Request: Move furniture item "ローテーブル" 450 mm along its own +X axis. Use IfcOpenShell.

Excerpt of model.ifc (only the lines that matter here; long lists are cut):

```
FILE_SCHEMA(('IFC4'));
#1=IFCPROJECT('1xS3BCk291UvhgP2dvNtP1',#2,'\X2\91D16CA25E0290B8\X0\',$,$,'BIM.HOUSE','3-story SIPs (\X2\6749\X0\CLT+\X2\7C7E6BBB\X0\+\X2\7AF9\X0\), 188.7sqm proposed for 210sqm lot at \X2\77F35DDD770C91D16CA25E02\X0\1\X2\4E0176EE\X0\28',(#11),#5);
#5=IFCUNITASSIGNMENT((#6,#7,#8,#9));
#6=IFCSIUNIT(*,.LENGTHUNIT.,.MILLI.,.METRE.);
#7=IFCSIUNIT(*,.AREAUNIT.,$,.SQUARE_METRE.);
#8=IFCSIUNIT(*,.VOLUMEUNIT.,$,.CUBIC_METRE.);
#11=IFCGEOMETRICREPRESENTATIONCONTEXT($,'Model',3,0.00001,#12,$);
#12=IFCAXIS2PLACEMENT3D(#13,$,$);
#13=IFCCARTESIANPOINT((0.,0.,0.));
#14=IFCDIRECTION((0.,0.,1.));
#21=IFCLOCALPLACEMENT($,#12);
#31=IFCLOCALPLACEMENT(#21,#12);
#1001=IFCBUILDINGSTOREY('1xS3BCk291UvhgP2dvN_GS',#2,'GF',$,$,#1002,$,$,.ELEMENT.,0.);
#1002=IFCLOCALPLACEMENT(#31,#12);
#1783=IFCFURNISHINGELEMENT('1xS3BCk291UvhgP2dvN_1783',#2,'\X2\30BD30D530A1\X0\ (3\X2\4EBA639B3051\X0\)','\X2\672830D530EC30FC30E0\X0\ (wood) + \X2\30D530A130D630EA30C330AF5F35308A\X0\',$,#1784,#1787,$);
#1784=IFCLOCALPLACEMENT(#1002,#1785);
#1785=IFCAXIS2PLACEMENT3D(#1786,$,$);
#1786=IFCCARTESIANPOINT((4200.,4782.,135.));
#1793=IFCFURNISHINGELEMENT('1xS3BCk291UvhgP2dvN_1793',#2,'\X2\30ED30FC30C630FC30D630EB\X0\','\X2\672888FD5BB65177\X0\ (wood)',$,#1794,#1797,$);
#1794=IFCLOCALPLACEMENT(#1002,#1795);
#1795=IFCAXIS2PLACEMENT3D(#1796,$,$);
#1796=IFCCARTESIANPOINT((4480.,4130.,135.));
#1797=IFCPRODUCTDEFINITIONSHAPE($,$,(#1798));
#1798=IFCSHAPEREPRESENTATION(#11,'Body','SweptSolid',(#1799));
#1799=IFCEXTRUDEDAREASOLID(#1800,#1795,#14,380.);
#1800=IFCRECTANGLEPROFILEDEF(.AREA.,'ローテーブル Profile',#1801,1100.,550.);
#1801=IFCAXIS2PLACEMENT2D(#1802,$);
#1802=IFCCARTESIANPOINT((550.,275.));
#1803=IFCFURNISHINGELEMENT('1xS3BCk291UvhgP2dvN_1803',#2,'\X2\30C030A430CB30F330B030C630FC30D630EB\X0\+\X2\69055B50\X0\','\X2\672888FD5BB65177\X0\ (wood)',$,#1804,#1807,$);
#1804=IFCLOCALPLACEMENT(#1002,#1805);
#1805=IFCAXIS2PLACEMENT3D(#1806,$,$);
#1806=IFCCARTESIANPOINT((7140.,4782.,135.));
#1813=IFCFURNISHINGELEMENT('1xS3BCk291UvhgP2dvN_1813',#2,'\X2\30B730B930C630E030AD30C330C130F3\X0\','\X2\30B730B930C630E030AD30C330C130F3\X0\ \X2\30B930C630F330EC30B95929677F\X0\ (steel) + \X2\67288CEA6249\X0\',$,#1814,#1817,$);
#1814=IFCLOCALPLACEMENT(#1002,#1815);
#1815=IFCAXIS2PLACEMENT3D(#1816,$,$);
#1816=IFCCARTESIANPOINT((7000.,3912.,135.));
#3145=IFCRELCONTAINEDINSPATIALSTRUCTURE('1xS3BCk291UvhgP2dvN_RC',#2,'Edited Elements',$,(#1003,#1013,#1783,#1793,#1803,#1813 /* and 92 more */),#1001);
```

```python
import ifcopenshell
import ifcopenshell.api.geometry
import ifcopenshell.util.placement

model = ifcopenshell.open("model.ifc")

item = model.by_guid("1xS3BCk291UvhgP2dvN_1793")
matrix = ifcopenshell.util.placement.get_local_placement(item.ObjectPlacement)
matrix[:3, 3] += matrix[:3, 0] * 450.0
ifcopenshell.api.geometry.edit_object_placement(model, product=item, matrix=matrix, is_si=False)

print(ifcopenshell.util.placement.get_local_placement(item.ObjectPlacement).round(3) + 0.0)

model.write("model-out.ifc")
```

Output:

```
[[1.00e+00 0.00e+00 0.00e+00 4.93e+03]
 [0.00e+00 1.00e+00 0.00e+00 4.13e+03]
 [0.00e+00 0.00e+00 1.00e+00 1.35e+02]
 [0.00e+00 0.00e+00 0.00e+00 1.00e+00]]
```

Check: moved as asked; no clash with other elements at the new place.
